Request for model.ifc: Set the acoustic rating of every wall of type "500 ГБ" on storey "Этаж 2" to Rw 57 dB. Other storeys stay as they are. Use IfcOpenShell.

First a look at what the model holds.

```python
import ifcopenshell
import ifcopenshell.util.element

model = ifcopenshell.open("model.ifc")
print(model.schema)
storey = next(s for s in model.by_type("IfcBuildingStorey") if s.Name == "Этаж 2")
walls = [e for e in ifcopenshell.util.element.get_decomposition(storey) if e.is_a("IfcWall")]
seen = {}
for e in walls:
    element_type = ifcopenshell.util.element.get_type(e)
    key = (element_type.Name if element_type != e and element_type else None, ifcopenshell.util.element.get_pset(e, "Pset_WallCommon", "AcousticRating"))
    seen[key] = seen.get(key, 0) + 1
for (name, value), count in sorted(seen.items(), key=str):
    print(count, "x", name, "|", value)
```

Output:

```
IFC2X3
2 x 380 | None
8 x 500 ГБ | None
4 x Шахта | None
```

```python
import ifcopenshell
import ifcopenshell.api.pset
import ifcopenshell.util.element

model = ifcopenshell.open("model.ifc")

storey = next(s for s in model.by_type("IfcBuildingStorey") if s.Name == "Этаж 2")
walls = [e for e in ifcopenshell.util.element.get_decomposition(storey) if e.is_a("IfcWall")]

count = 0
for e in walls:
    element_type = ifcopenshell.util.element.get_type(e)
    if element_type in (None, e) or element_type.Name != "500 ГБ":
        continue
    # add_pset returns the element's existing set when there is one.
    pset = ifcopenshell.api.pset.add_pset(model, product=e, name="Pset_WallCommon")
    ifcopenshell.api.pset.edit_pset(model, pset=pset, properties={"AcousticRating": "Rw 57 dB"})
    count += 1

print(count, "walls updated")

model.write("model_edited.ifc")
```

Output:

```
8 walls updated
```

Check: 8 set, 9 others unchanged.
